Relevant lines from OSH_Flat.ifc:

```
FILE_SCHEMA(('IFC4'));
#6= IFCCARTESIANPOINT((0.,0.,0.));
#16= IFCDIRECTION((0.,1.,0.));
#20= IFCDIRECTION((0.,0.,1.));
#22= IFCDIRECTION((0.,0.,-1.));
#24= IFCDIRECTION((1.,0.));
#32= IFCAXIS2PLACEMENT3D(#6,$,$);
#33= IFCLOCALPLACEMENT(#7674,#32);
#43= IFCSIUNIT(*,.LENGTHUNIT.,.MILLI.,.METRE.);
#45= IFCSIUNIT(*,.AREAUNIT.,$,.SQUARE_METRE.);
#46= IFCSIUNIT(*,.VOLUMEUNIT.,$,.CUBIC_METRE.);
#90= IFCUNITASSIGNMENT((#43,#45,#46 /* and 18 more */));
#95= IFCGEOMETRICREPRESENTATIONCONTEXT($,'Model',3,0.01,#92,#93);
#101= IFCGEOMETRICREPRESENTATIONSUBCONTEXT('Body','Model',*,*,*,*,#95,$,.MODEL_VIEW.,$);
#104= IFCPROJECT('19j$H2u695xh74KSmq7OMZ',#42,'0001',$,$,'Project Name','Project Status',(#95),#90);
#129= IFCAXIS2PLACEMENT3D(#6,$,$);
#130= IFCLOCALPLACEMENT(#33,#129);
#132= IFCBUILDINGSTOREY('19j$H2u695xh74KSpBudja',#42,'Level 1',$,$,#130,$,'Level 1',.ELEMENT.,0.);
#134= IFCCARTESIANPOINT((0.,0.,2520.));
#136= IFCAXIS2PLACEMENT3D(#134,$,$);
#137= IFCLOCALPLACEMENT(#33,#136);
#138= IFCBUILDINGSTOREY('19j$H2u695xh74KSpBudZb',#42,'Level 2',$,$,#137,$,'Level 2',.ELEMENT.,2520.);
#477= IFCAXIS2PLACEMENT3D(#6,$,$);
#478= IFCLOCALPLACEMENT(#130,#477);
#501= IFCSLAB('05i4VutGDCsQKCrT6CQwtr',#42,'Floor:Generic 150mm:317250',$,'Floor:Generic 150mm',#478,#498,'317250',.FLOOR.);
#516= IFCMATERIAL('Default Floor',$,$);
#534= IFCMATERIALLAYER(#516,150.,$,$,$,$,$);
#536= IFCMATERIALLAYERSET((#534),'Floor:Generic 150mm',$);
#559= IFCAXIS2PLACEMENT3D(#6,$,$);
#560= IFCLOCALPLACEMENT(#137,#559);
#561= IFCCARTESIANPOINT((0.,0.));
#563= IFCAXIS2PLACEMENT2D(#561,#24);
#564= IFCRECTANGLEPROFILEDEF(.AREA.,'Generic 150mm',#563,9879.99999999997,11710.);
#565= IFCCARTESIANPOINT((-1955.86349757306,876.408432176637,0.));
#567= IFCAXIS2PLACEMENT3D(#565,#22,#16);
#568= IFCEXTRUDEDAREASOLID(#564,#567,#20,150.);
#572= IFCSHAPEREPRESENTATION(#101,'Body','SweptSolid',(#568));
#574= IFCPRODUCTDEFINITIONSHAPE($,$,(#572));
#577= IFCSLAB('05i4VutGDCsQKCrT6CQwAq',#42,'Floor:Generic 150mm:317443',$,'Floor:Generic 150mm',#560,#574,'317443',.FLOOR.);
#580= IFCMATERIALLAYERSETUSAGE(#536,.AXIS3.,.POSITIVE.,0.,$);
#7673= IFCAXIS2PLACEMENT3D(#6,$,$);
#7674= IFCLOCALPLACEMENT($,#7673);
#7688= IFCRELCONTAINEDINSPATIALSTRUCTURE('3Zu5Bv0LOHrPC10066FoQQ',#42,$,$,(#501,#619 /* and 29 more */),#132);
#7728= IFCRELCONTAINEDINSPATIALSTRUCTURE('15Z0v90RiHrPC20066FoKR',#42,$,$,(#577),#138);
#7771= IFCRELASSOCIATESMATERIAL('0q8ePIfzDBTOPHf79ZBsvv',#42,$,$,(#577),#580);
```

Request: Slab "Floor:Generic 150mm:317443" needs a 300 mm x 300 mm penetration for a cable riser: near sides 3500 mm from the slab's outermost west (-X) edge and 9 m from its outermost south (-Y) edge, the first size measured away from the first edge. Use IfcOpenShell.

```python
import numpy as np
import ifcopenshell
import ifcopenshell.api.feature
import ifcopenshell.api.geometry
import ifcopenshell.api.root
import ifcopenshell.geom
import ifcopenshell.util.placement
import ifcopenshell.util.representation
import ifcopenshell.util.shape
import ifcopenshell.util.unit

model = ifcopenshell.open("OSH_Flat.ifc")
unit_scale = ifcopenshell.util.unit.calculate_unit_scale(model)
settings = ifcopenshell.geom.settings()


def volume(element):
    """Net volume in cubic metres, openings subtracted."""
    shape = ifcopenshell.geom.create_shape(settings, element)
    return ifcopenshell.util.shape.get_volume(shape.geometry)


slab = model.by_guid("05i4VutGDCsQKCrT6CQwAq")
before = volume(slab)

# Extent in the slab's own axes, in metres. The edges named are its -X and -Y sides.
slab_shape = ifcopenshell.geom.create_shape(settings, slab)
vertices = ifcopenshell.util.shape.get_vertices(slab_shape.geometry)
x_min, y_min, bottom = vertices.min(axis=0)
top = vertices[:, 2].max()

opening = ifcopenshell.api.root.create_entity(model, ifc_class="IfcOpeningElement", name="Cable riser opening", predefined_type="OPENING")
context = ifcopenshell.util.representation.get_context(model, "Model", "Body", "MODEL_VIEW")
width, depth = 0.3, 0.3
outline = [(0.0, 0.0), (width, 0.0), (width, depth), (0.0, depth), (0.0, 0.0)]
# Overshoot both faces by 50 mm so the cut is clean.
shape = ifcopenshell.api.geometry.add_slab_representation(
    model, context=context, depth=top - bottom + 0.1, polyline=outline
)
ifcopenshell.api.geometry.assign_representation(model, product=opening, representation=shape)

matrix = ifcopenshell.util.placement.get_local_placement(slab.ObjectPlacement)
matrix[:, 3] = matrix @ np.append(np.array([x_min + 3.5, y_min + 9, bottom - 0.05]) / unit_scale, 1.0)
ifcopenshell.api.geometry.edit_object_placement(model, product=opening, matrix=matrix, is_si=False)
ifcopenshell.api.feature.add_feature(model, feature=opening, element=slab)

after = volume(slab)

print(f"slab volume {before:.3f} -> {after:.3f} m3")

model.write("OSH_Flat-out.ifc")
```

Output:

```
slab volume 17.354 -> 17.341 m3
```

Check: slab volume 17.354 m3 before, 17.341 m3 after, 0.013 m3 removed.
